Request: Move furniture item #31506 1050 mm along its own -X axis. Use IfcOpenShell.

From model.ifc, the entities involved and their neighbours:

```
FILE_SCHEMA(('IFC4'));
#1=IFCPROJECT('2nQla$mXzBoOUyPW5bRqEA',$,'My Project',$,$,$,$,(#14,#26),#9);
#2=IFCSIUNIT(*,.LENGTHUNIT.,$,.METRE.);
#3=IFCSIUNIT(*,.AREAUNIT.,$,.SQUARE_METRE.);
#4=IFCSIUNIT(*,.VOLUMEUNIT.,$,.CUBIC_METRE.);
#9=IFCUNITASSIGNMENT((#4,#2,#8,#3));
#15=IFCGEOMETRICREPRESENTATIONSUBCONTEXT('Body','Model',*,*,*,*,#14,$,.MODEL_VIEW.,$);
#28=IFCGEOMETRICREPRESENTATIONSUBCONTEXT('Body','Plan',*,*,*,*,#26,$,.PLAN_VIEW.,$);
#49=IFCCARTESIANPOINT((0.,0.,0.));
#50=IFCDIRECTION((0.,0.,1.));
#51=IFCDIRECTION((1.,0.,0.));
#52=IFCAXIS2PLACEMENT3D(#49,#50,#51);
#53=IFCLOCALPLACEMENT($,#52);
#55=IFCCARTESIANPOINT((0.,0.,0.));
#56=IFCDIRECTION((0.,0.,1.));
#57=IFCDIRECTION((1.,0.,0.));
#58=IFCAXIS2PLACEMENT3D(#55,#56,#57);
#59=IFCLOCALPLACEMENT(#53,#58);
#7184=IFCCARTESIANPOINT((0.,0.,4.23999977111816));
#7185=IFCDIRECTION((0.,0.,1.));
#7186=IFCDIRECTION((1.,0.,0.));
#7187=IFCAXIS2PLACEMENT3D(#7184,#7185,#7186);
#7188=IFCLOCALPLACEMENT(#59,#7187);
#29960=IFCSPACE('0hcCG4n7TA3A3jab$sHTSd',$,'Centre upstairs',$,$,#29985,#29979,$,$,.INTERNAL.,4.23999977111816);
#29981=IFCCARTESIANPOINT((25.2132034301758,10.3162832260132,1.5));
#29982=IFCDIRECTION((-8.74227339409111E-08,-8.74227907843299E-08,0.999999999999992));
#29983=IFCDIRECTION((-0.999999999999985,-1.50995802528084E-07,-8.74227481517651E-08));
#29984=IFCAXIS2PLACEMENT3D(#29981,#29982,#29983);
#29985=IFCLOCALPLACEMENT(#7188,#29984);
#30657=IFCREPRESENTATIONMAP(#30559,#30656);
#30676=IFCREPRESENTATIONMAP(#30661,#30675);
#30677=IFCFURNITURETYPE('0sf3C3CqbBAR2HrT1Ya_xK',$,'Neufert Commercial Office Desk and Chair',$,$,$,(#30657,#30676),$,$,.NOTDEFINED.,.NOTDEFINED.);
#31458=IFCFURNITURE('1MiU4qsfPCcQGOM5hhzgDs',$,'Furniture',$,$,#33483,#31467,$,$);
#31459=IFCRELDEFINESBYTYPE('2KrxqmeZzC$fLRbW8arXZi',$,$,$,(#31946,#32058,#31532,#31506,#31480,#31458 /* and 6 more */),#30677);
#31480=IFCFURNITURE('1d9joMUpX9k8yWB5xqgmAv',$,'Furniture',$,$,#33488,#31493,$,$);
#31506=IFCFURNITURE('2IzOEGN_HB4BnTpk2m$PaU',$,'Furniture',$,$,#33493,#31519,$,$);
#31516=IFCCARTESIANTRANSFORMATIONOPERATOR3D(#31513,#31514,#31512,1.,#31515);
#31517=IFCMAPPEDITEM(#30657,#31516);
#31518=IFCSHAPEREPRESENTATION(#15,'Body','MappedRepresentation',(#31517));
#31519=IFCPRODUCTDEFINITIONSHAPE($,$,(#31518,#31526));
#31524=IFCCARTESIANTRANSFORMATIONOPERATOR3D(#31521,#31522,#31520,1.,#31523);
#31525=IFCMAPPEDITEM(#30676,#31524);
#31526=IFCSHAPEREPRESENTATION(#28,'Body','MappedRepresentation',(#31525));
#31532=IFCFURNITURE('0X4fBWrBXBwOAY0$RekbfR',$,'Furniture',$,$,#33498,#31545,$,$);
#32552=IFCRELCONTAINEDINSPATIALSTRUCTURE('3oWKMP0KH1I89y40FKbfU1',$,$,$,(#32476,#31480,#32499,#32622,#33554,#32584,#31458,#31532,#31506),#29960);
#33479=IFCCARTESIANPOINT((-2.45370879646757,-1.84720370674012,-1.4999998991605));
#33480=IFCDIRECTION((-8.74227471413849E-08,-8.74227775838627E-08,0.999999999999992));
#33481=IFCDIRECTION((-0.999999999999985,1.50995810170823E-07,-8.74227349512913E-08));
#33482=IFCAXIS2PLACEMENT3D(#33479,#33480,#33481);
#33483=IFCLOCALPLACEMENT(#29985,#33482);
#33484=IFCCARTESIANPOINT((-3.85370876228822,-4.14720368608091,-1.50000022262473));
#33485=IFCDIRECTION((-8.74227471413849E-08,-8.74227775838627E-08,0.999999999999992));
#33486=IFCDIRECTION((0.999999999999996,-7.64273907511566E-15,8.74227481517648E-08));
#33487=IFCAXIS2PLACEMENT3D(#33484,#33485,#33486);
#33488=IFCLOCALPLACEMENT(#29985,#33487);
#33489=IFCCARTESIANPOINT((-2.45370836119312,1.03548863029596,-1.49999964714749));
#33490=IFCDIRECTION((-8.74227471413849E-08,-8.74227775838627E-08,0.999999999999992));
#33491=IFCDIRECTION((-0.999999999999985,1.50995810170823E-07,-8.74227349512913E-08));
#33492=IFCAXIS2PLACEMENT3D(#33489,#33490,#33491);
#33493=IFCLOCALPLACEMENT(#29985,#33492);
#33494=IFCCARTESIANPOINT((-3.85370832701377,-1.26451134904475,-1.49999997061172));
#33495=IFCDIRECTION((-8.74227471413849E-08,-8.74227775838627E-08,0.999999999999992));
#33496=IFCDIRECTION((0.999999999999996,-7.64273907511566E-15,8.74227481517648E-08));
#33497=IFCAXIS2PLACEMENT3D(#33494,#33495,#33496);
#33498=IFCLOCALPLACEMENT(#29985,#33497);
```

```python
import ifcopenshell
import ifcopenshell.api.geometry
import ifcopenshell.util.placement

model = ifcopenshell.open("model.ifc")

item = model.by_guid("2IzOEGN_HB4BnTpk2m$PaU")
matrix = ifcopenshell.util.placement.get_local_placement(item.ObjectPlacement)
matrix[:3, 3] -= matrix[:3, 0] * 1.05
ifcopenshell.api.geometry.edit_object_placement(model, product=item, matrix=matrix, is_si=False)

print(ifcopenshell.util.placement.get_local_placement(item.ObjectPlacement).round(3) + 0.0)

model.write("model_v2.ifc")
```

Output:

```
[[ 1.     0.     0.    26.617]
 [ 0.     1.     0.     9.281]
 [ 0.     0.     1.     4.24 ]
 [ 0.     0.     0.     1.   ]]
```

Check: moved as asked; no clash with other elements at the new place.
